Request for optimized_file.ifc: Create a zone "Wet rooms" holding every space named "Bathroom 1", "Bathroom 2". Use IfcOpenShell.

First a look at what the model holds.

```python
import ifcopenshell

model = ifcopenshell.open("optimized_file.ifc")
print(model.schema)
seen = {}
for space in model.by_type("IfcSpace"):
    seen[space.LongName] = seen.get(space.LongName, 0) + 1
for name, count in sorted(seen.items(), key=str):
    print(count, "x", name)
print("zones:", [z.Name for z in model.by_type("IfcZone")][:20])
```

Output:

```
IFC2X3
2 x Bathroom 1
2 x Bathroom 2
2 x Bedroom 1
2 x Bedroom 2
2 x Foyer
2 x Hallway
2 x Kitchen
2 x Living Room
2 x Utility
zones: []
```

```python
import ifcopenshell
import ifcopenshell.api.group
import ifcopenshell.api.root

model = ifcopenshell.open("optimized_file.ifc")

names = {"Bathroom 1", "Bathroom 2"}
spaces = [s for s in model.by_type("IfcSpace") if s.LongName in names]

zone = ifcopenshell.api.root.create_entity(model, ifc_class="IfcZone", name="Wet rooms")
ifcopenshell.api.group.assign_group(model, products=spaces, group=zone)
print(len(spaces), "spaces in", zone.Name)

model.write("optimized_file_updated.ifc")
```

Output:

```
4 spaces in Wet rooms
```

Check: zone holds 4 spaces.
